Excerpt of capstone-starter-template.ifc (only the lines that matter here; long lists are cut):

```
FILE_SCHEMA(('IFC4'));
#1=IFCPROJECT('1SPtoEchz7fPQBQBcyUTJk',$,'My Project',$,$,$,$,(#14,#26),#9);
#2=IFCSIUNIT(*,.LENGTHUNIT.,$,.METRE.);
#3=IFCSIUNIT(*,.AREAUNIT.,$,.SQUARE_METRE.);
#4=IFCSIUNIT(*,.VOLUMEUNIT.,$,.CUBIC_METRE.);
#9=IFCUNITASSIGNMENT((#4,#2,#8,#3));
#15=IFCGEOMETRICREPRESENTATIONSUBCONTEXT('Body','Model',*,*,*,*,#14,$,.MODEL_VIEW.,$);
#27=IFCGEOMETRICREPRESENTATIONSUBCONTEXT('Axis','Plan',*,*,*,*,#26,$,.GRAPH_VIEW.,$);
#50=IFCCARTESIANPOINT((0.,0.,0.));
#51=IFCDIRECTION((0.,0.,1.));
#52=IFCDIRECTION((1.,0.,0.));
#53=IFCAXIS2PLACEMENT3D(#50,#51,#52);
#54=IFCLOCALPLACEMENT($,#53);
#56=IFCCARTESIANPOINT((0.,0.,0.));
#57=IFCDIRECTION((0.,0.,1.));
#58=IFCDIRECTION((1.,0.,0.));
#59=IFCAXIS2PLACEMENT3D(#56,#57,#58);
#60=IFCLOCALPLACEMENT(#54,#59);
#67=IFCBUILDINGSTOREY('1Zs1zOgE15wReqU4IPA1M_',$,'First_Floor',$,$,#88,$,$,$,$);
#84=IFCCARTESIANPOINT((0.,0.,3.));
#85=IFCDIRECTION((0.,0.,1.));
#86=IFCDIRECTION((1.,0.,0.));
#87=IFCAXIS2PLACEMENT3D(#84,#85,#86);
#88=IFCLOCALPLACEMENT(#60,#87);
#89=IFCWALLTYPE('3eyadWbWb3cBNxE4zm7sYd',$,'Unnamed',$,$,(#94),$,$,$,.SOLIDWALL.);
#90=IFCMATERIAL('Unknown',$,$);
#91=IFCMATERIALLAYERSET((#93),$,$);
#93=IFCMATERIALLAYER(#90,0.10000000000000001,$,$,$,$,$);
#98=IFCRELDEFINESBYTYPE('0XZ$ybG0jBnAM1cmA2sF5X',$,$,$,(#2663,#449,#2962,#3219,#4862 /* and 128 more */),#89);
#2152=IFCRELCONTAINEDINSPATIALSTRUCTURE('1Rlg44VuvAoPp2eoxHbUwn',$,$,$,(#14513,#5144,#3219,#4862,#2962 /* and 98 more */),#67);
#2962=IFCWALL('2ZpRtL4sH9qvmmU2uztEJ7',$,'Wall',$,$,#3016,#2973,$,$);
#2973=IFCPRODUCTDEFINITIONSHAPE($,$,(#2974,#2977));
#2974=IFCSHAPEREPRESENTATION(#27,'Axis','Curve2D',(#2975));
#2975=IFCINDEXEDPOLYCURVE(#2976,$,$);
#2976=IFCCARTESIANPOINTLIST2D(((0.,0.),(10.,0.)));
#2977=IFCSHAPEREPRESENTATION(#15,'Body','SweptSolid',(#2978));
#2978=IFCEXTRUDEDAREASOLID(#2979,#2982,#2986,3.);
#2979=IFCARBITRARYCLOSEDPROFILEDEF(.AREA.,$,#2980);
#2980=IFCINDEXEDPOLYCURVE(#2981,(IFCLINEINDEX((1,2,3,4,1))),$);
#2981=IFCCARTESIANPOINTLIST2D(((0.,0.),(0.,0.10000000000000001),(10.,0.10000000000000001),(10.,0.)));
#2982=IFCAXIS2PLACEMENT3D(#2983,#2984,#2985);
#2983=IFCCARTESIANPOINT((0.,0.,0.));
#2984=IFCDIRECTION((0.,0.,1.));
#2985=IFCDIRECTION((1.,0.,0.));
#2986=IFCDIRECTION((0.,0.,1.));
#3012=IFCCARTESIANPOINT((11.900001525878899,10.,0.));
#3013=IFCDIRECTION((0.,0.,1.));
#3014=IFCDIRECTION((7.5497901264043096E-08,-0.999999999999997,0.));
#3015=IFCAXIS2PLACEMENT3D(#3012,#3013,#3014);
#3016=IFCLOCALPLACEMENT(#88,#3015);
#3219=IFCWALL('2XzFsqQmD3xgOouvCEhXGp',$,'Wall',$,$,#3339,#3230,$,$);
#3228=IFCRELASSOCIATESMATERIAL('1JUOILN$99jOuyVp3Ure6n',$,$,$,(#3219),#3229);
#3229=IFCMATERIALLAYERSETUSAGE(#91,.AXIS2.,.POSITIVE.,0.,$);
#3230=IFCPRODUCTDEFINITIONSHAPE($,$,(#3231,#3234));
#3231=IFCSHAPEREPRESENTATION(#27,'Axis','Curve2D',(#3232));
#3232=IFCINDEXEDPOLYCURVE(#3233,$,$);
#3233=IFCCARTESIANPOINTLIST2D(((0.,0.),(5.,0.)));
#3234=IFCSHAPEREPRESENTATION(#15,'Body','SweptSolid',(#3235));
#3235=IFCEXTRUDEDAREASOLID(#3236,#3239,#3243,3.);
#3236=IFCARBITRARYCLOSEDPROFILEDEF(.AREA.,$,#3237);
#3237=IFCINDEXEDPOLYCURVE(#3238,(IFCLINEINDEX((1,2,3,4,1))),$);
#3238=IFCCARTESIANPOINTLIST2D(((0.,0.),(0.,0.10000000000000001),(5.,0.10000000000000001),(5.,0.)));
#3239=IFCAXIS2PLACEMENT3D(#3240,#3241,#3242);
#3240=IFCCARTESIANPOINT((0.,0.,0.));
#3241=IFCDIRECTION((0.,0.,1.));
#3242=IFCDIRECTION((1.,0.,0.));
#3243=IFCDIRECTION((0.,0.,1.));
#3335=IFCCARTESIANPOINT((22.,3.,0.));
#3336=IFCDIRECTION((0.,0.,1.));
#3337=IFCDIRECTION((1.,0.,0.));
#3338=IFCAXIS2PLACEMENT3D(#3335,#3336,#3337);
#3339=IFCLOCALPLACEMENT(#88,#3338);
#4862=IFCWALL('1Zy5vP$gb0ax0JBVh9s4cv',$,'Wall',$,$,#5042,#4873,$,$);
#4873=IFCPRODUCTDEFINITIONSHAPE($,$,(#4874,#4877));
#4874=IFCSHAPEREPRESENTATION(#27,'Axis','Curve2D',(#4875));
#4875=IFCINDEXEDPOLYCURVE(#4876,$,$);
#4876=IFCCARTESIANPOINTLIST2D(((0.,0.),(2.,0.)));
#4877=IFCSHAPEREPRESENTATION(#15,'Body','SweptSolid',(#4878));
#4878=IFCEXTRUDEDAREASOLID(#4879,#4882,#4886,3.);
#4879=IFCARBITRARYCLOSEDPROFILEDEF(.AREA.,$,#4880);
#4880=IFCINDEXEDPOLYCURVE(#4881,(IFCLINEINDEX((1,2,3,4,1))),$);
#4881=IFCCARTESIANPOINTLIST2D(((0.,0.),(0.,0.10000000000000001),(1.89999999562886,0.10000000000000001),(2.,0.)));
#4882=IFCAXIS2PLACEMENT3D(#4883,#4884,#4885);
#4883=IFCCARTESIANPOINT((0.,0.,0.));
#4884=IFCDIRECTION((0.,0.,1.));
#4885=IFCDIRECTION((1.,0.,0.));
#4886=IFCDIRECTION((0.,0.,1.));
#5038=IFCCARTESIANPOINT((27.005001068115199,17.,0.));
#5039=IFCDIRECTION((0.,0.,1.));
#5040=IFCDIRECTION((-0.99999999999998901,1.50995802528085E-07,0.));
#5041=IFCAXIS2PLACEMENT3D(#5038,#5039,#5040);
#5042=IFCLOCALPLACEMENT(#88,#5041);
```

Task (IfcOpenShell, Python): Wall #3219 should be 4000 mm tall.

```python
import ifcopenshell
import ifcopenshell.geom
import ifcopenshell.util.representation
import ifcopenshell.util.shape

model = ifcopenshell.open("capstone-starter-template.ifc")
settings = ifcopenshell.geom.settings()


def volume(element):
    """Net volume in cubic metres, openings subtracted."""
    shape = ifcopenshell.geom.create_shape(settings, element)
    return ifcopenshell.util.shape.get_volume(shape.geometry)


wall = model.by_guid("2XzFsqQmD3xgOouvCEhXGp")
before = volume(wall)

body = ifcopenshell.util.representation.get_representation(wall, "Model", "Body")
solid = body.Items[0]
old_height = solid.Depth
solid.Depth = 4.0
after = volume(wall)

print(f"height {old_height:g} -> {solid.Depth:g}, volume {before:.3f} -> {after:.3f} m3")

model.write("capstone-starter-template_edited.ifc")
```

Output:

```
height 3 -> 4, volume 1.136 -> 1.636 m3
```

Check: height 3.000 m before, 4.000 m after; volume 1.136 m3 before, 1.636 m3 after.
